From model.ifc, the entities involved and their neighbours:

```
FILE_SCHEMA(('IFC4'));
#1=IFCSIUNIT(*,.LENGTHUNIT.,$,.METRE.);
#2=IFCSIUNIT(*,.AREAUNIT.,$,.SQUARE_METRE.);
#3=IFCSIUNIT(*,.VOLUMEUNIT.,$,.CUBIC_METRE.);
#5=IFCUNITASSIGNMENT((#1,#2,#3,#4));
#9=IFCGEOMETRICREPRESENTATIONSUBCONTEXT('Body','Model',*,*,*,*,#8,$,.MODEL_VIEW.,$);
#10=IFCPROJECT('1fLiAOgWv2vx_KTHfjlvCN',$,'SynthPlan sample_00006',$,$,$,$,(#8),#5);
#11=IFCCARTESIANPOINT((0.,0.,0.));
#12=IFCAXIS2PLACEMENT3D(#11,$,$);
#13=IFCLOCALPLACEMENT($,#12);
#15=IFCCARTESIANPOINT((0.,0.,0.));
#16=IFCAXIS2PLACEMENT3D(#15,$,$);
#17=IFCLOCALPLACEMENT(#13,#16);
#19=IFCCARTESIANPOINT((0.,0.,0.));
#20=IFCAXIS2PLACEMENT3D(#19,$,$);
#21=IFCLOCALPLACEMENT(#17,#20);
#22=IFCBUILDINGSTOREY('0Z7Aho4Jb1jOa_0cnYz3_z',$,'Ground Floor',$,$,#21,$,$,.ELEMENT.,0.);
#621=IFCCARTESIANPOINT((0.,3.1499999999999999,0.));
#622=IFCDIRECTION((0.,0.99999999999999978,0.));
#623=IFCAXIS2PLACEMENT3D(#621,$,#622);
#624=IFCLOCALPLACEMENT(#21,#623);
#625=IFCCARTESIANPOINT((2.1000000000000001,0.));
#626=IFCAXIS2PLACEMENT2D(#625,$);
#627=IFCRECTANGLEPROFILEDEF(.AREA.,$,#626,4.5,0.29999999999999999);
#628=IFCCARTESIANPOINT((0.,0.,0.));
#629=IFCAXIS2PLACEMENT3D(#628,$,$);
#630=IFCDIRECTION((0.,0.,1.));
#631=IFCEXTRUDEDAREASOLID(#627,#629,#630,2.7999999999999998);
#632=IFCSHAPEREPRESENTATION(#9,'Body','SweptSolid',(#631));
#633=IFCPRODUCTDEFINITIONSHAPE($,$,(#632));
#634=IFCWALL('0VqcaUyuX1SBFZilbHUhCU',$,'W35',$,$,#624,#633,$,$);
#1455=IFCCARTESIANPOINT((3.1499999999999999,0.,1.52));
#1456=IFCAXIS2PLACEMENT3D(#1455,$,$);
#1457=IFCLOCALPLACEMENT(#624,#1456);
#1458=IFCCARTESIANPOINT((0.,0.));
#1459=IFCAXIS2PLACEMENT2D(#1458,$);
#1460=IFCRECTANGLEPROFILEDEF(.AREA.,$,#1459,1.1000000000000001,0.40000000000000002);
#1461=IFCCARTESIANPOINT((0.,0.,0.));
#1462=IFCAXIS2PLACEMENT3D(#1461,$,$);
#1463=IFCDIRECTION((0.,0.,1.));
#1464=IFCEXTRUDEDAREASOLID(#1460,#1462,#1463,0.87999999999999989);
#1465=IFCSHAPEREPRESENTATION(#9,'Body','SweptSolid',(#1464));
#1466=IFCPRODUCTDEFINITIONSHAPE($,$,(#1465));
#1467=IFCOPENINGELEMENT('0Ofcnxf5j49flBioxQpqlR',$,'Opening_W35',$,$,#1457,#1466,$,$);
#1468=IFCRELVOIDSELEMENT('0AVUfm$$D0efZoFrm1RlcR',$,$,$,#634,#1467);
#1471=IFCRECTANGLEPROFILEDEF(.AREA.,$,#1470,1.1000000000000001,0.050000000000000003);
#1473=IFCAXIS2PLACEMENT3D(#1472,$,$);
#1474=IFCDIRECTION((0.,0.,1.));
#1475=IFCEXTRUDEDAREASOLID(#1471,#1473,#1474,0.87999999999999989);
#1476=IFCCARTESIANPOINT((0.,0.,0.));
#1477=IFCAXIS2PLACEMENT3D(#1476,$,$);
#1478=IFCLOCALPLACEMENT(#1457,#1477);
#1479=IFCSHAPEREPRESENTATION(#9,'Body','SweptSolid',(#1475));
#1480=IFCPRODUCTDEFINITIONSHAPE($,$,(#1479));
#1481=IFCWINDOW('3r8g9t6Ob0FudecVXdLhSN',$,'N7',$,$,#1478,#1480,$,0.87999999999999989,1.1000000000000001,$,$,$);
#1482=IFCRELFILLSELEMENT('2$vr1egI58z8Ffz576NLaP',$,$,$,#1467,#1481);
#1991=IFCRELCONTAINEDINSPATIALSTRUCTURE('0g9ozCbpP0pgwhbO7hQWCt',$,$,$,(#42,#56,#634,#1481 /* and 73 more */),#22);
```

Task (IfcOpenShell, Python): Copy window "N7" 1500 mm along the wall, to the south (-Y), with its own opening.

```python
import ifcopenshell
import ifcopenshell.api.feature
import ifcopenshell.api.geometry
import ifcopenshell.api.root
import ifcopenshell.geom
import ifcopenshell.util.element
import ifcopenshell.util.placement
import ifcopenshell.util.shape

model = ifcopenshell.open("model.ifc")
settings = ifcopenshell.geom.settings()


def volume(element):
    """Net volume in cubic metres, openings subtracted."""
    shape = ifcopenshell.geom.create_shape(settings, element)
    return ifcopenshell.util.shape.get_volume(shape.geometry)


window = model.by_guid("3r8g9t6Ob0FudecVXdLhSN")
opening = window.FillsVoids[0].RelatingOpeningElement
wall = opening.VoidsElements[0].RelatingBuildingElement
before = volume(wall)
shift = ifcopenshell.util.placement.get_local_placement(wall.ObjectPlacement)[:3, 0] * -1.5

# copy_class copies the void relationship, type, container and properties, but no geometry.
new_opening = ifcopenshell.api.root.copy_class(model, product=opening)
new_opening.Representation = ifcopenshell.util.element.copy_deep(
    model, opening.Representation, exclude=["IfcGeometricRepresentationContext", "IfcRepresentationMap"]
)
new_window = ifcopenshell.api.root.copy_class(model, product=window)
new_window.Representation = ifcopenshell.util.element.copy_deep(
    model, window.Representation, exclude=["IfcGeometricRepresentationContext", "IfcRepresentationMap"]
)
ifcopenshell.api.feature.add_filling(model, opening=new_opening, element=new_window)

for old, new in ((opening, new_opening), (window, new_window)):
    matrix = ifcopenshell.util.placement.get_local_placement(old.ObjectPlacement)
    matrix[:3, 3] += shift
    ifcopenshell.api.geometry.edit_object_placement(model, product=new, matrix=matrix, is_si=False)

after = volume(wall)

print(f"wall volume {before:.3f} -> {after:.3f} m3")

model.write("model_rev.ifc")
```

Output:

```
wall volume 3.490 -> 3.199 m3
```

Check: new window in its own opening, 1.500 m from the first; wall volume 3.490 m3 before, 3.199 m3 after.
